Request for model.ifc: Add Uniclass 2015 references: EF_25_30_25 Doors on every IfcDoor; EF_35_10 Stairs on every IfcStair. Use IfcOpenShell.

First a look at what the model holds.

```python
import ifcopenshell

model = ifcopenshell.open("model.ifc")
print(model.schema)
print("classifications:", [c.Name for c in model.by_type("IfcClassification")])
for ifc_class in ("IfcDoor", "IfcRoof", "IfcStair", "IfcWall", "IfcWindow"):
    print(ifc_class, len(model.by_type(ifc_class)))
```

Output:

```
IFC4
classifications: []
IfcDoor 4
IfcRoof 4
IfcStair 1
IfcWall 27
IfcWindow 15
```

```python
import ifcopenshell
import ifcopenshell.api.classification

model = ifcopenshell.open("model.ifc")

system = ifcopenshell.api.classification.add_classification(model, classification="Uniclass 2015")

codes = {
    "IfcDoor": ("EF_25_30_25", "Doors"),
    "IfcStair": ("EF_35_10", "Stairs"),
}
for ifc_class, (code, name) in codes.items():
    products = model.by_type(ifc_class)
    ifcopenshell.api.classification.add_reference(
        model, products=products, classification=system, identification=code, name=name
    )
    print(code, len(products))

model.write("model_rev.ifc")
```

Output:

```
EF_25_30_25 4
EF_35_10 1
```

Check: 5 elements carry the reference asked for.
